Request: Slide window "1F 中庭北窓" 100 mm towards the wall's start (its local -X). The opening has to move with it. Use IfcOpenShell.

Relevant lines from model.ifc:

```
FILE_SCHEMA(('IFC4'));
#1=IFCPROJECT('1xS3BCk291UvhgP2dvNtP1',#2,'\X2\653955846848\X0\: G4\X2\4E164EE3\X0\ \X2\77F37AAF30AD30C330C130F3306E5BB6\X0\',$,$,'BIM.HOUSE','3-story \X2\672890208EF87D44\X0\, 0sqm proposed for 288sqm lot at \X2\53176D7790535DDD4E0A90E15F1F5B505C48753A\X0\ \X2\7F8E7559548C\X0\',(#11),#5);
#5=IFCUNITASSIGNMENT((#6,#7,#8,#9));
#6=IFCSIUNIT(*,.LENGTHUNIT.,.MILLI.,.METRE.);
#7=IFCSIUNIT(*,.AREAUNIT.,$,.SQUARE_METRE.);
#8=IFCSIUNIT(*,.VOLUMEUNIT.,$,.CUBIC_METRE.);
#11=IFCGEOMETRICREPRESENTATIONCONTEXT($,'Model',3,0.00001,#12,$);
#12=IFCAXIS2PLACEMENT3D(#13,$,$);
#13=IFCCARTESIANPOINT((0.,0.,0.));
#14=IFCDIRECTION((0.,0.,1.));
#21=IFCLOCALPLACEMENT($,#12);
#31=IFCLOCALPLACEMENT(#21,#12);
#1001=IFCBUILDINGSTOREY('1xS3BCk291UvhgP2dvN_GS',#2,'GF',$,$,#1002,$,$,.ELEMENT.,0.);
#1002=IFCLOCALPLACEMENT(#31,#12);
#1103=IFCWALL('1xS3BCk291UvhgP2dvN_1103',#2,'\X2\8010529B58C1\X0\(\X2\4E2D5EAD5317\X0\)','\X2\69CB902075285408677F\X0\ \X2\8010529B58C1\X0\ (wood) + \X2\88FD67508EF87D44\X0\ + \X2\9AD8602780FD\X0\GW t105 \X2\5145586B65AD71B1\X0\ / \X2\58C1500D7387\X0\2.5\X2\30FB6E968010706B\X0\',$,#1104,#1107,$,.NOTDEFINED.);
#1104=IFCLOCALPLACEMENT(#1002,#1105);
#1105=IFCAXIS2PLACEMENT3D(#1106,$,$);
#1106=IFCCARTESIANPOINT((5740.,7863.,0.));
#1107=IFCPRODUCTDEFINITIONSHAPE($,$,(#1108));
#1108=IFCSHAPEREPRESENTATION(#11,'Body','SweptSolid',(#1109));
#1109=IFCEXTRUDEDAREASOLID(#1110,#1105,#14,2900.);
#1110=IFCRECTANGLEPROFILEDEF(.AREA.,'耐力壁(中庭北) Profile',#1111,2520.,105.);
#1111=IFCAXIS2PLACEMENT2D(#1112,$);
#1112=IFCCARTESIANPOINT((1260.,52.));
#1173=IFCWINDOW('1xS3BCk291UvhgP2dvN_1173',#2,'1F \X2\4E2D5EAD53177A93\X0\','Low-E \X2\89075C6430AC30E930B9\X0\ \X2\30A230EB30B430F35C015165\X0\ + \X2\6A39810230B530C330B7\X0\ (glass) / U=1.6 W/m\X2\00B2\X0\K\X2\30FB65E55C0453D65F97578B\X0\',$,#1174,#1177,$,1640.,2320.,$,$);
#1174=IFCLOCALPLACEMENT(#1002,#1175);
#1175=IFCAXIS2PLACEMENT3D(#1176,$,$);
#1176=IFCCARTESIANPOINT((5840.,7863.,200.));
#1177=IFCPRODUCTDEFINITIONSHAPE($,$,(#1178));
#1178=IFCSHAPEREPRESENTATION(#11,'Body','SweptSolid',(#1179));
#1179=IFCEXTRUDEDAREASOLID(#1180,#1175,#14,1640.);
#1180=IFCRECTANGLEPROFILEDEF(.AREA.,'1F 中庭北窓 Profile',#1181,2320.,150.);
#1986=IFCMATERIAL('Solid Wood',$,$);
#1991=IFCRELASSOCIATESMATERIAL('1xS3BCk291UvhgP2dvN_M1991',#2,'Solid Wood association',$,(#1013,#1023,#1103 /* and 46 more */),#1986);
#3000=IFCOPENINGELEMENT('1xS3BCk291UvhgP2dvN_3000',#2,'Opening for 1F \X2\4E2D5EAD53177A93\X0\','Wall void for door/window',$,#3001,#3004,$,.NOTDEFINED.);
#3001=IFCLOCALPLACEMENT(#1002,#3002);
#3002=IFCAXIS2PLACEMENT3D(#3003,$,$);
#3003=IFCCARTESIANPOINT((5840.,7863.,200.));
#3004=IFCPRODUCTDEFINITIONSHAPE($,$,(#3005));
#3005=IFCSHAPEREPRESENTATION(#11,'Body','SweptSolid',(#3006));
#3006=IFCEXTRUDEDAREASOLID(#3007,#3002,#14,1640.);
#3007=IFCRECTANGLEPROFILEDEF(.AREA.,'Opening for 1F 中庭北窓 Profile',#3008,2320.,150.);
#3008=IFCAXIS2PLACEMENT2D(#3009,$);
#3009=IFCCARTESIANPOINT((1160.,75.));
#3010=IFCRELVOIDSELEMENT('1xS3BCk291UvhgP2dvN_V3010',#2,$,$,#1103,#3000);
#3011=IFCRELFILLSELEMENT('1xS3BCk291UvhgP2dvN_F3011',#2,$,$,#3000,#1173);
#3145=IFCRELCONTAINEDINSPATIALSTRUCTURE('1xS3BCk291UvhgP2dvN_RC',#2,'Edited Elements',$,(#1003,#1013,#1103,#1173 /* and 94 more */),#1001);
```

```python
import ifcopenshell
import ifcopenshell.api.geometry
import ifcopenshell.util.placement
import ifcopenshell.util.unit

model = ifcopenshell.open("model.ifc")
unit_scale = ifcopenshell.util.unit.calculate_unit_scale(model)

window = model.by_guid("1xS3BCk291UvhgP2dvN_1173")
opening = window.FillsVoids[0].RelatingOpeningElement
wall = opening.VoidsElements[0].RelatingBuildingElement

wall_matrix = ifcopenshell.util.placement.get_local_placement(wall.ObjectPlacement)
shift = wall_matrix[:3, 0] * -0.1 / unit_scale
before = ifcopenshell.util.placement.get_local_placement(window.ObjectPlacement)[:3, 3].copy()

# The window is not placed relative to its opening, so move both.
for product in (opening, window):
    matrix = ifcopenshell.util.placement.get_local_placement(product.ObjectPlacement)
    matrix[:3, 3] += shift
    ifcopenshell.api.geometry.edit_object_placement(model, product=product, matrix=matrix, is_si=False)

after = ifcopenshell.util.placement.get_local_placement(window.ObjectPlacement)[:3, 3]
print("window moved by", (after - before).round(3) + 0.0)

model.write("model_edited.ifc")
```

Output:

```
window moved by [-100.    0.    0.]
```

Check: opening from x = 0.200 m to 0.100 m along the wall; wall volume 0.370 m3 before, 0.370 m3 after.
